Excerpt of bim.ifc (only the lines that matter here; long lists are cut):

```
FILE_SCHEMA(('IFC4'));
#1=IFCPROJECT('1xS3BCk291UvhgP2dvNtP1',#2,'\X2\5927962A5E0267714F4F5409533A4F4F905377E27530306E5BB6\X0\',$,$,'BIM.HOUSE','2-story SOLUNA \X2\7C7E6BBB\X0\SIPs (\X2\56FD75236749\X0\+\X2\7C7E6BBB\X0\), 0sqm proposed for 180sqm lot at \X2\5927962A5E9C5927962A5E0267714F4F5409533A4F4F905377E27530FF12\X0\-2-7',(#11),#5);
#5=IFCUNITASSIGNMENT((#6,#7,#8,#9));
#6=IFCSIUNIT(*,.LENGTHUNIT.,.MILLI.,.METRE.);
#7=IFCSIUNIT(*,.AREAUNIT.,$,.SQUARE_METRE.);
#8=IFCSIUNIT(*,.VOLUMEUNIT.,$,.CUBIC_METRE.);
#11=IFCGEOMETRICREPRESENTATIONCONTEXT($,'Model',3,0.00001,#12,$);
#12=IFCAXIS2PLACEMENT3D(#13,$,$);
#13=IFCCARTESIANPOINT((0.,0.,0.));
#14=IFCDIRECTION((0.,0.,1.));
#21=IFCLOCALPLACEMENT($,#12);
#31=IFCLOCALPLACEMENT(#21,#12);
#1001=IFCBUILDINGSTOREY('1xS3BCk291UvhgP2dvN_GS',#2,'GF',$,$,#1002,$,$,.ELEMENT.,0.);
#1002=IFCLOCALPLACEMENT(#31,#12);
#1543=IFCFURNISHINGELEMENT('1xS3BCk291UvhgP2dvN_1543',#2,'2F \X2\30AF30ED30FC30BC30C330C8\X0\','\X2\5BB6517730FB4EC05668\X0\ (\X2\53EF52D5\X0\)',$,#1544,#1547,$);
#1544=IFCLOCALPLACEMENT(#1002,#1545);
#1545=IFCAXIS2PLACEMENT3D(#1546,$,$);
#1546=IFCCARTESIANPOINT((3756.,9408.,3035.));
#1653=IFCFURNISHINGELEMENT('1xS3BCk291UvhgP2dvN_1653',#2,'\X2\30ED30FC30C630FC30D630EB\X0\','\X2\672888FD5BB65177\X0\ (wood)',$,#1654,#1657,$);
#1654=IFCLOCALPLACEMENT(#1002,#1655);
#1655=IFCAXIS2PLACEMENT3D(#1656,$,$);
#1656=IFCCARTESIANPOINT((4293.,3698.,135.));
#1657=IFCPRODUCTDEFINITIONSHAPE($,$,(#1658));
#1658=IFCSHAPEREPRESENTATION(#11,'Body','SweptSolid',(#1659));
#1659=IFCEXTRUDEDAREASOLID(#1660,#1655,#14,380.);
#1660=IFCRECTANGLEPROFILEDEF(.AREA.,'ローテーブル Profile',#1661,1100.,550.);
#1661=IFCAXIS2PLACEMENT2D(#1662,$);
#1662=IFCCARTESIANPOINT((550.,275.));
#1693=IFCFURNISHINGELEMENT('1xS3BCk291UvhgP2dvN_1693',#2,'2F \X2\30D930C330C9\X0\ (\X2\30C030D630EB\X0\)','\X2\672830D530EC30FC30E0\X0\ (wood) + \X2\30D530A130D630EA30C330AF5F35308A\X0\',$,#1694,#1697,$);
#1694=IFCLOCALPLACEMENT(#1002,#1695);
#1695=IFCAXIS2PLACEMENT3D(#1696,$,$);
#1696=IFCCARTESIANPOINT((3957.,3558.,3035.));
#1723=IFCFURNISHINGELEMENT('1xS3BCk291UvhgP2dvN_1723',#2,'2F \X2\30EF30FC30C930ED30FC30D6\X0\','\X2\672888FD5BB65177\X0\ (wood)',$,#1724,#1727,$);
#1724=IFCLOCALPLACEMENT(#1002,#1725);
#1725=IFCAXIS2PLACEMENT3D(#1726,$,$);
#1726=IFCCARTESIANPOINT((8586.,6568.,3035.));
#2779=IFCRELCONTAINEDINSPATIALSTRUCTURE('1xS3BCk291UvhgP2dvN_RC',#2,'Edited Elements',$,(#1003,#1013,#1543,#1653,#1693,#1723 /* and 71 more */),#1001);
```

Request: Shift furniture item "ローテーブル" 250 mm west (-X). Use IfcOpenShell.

```python
import ifcopenshell
import ifcopenshell.api.geometry
import ifcopenshell.util.placement

model = ifcopenshell.open("bim.ifc")

item = model.by_id(1653)
matrix = ifcopenshell.util.placement.get_local_placement(item.ObjectPlacement)
matrix[0, 3] -= 250.0
ifcopenshell.api.geometry.edit_object_placement(model, product=item, matrix=matrix, is_si=False)

print(ifcopenshell.util.placement.get_local_placement(item.ObjectPlacement).round(3) + 0.0)

model.write("bim-out.ifc")
```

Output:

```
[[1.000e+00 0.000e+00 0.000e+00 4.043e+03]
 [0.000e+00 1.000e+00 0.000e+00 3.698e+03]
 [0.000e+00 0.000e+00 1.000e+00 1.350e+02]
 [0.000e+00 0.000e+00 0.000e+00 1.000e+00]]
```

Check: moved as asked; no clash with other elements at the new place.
